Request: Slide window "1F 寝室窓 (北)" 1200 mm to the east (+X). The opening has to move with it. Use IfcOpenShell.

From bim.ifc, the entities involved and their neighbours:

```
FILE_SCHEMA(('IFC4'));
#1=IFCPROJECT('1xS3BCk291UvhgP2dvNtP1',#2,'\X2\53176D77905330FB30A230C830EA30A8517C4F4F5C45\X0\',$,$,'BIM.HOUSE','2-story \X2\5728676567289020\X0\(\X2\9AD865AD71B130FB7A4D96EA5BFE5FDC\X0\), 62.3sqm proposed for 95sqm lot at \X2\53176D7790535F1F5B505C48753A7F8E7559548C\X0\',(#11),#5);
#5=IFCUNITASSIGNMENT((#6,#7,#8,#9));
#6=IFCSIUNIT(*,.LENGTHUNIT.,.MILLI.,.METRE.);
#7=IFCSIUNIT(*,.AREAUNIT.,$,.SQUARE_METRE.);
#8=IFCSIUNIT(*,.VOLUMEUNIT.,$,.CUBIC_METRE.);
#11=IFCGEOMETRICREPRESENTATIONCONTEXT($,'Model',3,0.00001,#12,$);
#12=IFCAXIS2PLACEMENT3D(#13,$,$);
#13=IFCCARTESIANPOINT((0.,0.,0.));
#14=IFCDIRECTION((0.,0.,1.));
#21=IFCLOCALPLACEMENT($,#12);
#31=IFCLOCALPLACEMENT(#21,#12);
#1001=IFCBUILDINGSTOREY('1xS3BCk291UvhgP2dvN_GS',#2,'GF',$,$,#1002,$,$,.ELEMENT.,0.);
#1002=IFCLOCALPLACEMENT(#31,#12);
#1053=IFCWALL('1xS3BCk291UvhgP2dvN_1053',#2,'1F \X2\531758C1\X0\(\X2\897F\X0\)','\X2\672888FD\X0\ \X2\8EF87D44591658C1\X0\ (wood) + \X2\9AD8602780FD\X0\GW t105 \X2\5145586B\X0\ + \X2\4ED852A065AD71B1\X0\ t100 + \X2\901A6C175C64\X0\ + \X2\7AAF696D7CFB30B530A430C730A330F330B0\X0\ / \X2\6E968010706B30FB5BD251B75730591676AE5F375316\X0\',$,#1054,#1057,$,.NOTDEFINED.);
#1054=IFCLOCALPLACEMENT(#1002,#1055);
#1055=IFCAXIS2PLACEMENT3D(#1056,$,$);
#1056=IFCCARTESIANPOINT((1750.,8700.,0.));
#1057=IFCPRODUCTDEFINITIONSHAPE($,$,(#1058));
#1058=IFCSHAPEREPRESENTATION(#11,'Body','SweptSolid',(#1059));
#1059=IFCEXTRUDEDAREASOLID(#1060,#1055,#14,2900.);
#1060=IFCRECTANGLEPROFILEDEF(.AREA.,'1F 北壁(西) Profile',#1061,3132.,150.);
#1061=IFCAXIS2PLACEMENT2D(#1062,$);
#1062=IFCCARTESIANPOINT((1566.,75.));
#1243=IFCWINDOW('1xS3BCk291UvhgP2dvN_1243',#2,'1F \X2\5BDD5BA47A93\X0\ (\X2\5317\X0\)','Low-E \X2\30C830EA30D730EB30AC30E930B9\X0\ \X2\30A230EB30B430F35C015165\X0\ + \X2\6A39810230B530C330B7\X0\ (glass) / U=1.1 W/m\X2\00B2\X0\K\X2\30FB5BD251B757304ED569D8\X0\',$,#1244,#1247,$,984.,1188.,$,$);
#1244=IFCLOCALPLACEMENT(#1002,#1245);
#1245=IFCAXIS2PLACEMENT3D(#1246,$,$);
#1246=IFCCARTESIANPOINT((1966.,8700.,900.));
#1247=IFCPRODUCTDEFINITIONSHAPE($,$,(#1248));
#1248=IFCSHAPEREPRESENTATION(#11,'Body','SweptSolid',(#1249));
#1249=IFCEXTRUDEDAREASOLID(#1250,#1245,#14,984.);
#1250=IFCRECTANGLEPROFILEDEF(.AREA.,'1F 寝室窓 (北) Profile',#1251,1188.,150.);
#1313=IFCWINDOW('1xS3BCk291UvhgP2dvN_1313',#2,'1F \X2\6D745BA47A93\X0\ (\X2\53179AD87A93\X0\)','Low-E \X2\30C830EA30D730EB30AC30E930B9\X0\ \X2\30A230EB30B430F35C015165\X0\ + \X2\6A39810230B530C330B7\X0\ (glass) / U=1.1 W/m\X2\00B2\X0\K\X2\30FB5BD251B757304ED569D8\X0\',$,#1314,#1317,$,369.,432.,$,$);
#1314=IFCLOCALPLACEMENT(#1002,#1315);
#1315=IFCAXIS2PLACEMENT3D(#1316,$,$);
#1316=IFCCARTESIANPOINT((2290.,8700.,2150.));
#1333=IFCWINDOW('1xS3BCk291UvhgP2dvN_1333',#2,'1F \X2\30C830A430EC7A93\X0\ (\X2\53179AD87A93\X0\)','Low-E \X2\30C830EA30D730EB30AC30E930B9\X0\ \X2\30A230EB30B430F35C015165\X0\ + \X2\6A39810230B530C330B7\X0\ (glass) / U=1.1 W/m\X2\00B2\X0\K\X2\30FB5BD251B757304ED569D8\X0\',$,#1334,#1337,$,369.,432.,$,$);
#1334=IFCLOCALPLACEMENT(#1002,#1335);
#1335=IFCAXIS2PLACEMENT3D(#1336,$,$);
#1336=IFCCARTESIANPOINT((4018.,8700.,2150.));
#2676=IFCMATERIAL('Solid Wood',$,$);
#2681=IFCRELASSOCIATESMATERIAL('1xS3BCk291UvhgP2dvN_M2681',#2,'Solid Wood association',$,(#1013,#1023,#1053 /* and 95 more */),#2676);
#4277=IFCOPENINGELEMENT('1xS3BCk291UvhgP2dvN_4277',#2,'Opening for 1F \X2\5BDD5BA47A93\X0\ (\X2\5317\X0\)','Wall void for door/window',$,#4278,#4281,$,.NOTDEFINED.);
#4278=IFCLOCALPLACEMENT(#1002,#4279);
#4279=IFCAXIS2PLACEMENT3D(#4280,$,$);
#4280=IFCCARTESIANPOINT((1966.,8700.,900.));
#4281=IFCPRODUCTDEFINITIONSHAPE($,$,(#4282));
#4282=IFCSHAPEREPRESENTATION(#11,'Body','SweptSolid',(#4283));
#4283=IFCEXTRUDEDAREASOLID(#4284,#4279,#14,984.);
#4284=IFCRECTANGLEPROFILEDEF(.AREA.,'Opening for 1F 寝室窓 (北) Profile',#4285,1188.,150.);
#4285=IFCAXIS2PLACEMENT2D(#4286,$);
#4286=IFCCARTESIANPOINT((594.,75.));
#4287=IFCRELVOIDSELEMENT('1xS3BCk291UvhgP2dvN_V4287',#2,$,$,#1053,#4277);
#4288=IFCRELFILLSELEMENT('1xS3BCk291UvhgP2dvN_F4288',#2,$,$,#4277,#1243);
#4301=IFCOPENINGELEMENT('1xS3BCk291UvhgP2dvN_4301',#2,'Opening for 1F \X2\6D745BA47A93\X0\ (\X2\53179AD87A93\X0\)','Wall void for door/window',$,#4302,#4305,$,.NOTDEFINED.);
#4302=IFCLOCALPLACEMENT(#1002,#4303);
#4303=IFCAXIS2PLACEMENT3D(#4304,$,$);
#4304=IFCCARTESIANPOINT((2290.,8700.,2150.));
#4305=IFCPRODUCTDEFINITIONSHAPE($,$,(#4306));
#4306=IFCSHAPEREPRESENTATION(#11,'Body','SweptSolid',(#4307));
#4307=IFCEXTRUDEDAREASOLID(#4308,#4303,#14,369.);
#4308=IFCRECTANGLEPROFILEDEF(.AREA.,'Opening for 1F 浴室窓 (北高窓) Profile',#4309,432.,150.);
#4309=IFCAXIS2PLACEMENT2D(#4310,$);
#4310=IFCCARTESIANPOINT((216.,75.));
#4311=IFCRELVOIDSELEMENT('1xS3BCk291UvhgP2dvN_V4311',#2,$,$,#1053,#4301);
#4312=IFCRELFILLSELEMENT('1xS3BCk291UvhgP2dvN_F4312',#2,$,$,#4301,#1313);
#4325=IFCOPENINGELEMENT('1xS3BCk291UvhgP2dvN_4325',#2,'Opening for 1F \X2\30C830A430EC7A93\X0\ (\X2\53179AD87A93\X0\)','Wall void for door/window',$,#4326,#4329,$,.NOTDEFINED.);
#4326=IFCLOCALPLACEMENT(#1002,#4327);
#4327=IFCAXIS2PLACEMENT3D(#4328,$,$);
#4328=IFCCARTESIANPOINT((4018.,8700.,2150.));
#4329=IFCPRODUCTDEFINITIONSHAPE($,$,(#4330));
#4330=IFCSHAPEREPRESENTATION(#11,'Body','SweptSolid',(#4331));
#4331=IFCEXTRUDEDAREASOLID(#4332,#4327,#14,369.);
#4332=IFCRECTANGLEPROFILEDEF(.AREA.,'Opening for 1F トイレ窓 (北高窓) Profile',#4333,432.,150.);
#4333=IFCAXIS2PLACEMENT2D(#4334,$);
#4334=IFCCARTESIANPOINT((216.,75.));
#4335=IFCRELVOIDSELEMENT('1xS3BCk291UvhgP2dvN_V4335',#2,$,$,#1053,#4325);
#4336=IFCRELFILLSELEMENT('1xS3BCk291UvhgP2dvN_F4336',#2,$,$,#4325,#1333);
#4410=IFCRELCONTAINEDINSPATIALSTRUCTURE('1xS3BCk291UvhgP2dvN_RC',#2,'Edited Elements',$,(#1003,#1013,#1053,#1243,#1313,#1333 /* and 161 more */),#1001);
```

```python
import ifcopenshell
import ifcopenshell.api.geometry
import ifcopenshell.util.placement
import ifcopenshell.util.unit

model = ifcopenshell.open("bim.ifc")
unit_scale = ifcopenshell.util.unit.calculate_unit_scale(model)

window = model.by_guid("1xS3BCk291UvhgP2dvN_1243")
opening = window.FillsVoids[0].RelatingOpeningElement
wall = opening.VoidsElements[0].RelatingBuildingElement

wall_matrix = ifcopenshell.util.placement.get_local_placement(wall.ObjectPlacement)
shift = wall_matrix[:3, 0] * 1.2 / unit_scale
before = ifcopenshell.util.placement.get_local_placement(window.ObjectPlacement)[:3, 3].copy()

# The window is not placed relative to its opening, so move both.
for product in (opening, window):
    matrix = ifcopenshell.util.placement.get_local_placement(product.ObjectPlacement)
    matrix[:3, 3] += shift
    ifcopenshell.api.geometry.edit_object_placement(model, product=product, matrix=matrix, is_si=False)

after = ifcopenshell.util.placement.get_local_placement(window.ObjectPlacement)[:3, 3]
print("window moved by", (after - before).round(3) + 0.0)

model.write("bim_rev.ifc")
```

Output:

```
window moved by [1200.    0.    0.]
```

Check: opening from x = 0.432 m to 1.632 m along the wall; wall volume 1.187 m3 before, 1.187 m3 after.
